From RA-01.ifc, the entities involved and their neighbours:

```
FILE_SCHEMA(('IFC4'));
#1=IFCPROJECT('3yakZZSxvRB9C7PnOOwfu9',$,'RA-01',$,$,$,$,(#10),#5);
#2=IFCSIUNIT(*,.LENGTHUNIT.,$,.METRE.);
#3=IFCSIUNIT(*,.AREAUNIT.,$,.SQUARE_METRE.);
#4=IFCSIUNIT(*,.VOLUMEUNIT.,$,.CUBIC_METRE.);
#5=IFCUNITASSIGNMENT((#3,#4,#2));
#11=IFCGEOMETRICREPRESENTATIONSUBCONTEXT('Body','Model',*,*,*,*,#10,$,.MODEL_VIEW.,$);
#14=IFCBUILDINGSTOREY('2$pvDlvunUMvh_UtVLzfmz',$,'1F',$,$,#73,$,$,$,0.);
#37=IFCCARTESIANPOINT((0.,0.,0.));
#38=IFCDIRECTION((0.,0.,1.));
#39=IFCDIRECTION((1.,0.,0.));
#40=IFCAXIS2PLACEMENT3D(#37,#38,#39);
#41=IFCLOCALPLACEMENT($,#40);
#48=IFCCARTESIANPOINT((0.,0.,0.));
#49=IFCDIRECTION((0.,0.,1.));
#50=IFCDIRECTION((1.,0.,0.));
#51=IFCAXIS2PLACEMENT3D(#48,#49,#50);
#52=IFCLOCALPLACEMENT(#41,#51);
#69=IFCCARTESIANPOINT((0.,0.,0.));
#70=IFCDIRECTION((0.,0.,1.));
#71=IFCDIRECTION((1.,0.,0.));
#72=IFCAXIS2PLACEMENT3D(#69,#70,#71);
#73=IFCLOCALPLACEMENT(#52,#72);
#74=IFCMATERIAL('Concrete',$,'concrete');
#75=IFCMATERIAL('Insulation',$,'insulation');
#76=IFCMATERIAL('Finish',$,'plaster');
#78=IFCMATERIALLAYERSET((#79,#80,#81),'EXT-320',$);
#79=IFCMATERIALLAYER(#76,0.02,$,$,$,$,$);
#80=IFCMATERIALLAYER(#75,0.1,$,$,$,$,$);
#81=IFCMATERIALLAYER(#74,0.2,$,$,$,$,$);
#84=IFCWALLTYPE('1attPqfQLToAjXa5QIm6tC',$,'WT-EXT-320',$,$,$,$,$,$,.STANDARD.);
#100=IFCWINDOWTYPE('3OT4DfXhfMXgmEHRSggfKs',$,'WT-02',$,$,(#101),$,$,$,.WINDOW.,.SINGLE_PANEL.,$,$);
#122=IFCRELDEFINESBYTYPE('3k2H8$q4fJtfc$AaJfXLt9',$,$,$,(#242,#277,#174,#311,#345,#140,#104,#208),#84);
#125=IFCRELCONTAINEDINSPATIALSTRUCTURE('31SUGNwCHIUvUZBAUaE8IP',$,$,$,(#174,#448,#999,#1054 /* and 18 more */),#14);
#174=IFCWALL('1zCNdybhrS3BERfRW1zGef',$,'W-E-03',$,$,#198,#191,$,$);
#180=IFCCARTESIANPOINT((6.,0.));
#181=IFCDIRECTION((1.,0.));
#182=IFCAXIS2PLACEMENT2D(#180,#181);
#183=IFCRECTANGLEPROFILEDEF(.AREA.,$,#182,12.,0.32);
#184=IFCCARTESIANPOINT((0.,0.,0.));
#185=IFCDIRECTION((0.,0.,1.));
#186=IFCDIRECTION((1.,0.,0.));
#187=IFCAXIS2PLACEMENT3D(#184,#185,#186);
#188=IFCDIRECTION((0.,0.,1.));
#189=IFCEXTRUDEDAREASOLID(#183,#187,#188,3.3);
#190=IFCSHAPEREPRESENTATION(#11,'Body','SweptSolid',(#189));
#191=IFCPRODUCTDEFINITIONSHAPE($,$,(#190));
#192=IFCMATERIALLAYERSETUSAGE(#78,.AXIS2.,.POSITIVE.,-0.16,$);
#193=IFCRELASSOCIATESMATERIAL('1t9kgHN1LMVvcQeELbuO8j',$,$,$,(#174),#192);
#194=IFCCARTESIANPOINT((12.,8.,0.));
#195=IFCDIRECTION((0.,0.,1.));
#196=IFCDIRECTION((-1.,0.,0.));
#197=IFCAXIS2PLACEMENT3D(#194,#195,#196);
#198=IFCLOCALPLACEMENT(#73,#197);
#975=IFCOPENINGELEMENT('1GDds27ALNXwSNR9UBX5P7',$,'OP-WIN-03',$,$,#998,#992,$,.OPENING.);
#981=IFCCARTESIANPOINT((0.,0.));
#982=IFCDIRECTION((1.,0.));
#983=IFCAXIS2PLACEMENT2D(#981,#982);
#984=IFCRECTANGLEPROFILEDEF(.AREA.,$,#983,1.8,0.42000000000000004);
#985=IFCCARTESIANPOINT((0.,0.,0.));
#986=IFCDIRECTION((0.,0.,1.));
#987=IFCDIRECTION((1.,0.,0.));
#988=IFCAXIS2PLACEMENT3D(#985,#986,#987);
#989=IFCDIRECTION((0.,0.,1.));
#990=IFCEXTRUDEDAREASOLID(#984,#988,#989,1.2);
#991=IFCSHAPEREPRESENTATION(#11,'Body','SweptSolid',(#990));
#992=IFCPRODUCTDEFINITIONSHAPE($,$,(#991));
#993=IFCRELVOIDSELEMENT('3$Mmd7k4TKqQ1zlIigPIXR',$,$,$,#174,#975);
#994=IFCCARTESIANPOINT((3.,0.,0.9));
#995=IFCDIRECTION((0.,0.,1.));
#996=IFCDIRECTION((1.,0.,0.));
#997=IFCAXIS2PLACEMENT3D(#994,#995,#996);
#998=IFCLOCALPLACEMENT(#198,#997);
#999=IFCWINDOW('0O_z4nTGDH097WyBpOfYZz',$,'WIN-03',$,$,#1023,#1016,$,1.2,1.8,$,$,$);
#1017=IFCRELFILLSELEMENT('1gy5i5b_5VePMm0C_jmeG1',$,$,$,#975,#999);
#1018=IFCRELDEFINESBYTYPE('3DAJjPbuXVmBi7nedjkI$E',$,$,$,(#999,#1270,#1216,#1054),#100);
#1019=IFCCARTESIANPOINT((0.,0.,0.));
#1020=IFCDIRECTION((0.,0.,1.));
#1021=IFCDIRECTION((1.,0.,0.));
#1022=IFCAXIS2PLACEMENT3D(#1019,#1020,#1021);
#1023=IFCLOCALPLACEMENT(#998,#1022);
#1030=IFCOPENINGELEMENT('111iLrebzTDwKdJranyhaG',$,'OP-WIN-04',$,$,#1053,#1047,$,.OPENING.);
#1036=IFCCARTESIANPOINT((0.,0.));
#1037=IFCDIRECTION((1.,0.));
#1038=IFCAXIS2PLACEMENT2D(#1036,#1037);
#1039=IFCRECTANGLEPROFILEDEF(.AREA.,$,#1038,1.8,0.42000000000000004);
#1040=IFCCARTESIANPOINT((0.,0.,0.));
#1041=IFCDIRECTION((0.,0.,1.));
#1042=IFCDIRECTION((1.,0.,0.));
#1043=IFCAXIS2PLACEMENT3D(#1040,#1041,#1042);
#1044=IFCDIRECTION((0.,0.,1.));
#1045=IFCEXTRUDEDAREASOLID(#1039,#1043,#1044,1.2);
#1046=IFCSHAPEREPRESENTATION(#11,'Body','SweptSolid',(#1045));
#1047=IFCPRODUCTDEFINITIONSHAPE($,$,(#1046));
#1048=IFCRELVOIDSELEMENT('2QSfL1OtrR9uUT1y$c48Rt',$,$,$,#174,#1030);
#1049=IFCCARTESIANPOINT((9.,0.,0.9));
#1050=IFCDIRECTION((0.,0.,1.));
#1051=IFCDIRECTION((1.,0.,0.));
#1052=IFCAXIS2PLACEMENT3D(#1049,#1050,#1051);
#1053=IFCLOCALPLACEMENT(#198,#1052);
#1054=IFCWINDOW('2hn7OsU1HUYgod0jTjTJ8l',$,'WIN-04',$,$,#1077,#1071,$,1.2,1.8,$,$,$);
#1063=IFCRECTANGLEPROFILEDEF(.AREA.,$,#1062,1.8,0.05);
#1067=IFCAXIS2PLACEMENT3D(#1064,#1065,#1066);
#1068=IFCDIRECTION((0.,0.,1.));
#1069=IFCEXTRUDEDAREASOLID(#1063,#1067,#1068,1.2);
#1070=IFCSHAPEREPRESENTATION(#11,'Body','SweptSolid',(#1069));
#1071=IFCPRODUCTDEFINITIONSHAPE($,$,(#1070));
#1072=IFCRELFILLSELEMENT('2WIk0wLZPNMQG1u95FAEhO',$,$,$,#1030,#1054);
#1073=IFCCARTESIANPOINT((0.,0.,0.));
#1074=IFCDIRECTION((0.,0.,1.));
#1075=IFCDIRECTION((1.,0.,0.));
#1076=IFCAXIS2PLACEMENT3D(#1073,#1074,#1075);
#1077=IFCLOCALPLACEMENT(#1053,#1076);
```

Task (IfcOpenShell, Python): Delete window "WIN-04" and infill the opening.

```python
import ifcopenshell
import ifcopenshell.api.feature
import ifcopenshell.api.root
import ifcopenshell.geom
import ifcopenshell.util.shape

model = ifcopenshell.open("RA-01.ifc")
settings = ifcopenshell.geom.settings()


def volume(element):
    """Net volume in cubic metres, openings subtracted."""
    shape = ifcopenshell.geom.create_shape(settings, element)
    return ifcopenshell.util.shape.get_volume(shape.geometry)


window = model.by_guid("2hn7OsU1HUYgod0jTjTJ8l")
opening = window.FillsVoids[0].RelatingOpeningElement
wall = opening.VoidsElements[0].RelatingBuildingElement
before = volume(wall)

ifcopenshell.api.root.remove_product(model, product=window)
ifcopenshell.api.feature.remove_feature(model, feature=opening)

after = volume(wall)

print(f"wall volume {before:.3f} -> {after:.3f} m3")

model.write("RA-01_rev.ifc")
```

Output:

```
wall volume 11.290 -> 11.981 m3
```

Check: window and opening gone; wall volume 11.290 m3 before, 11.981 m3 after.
